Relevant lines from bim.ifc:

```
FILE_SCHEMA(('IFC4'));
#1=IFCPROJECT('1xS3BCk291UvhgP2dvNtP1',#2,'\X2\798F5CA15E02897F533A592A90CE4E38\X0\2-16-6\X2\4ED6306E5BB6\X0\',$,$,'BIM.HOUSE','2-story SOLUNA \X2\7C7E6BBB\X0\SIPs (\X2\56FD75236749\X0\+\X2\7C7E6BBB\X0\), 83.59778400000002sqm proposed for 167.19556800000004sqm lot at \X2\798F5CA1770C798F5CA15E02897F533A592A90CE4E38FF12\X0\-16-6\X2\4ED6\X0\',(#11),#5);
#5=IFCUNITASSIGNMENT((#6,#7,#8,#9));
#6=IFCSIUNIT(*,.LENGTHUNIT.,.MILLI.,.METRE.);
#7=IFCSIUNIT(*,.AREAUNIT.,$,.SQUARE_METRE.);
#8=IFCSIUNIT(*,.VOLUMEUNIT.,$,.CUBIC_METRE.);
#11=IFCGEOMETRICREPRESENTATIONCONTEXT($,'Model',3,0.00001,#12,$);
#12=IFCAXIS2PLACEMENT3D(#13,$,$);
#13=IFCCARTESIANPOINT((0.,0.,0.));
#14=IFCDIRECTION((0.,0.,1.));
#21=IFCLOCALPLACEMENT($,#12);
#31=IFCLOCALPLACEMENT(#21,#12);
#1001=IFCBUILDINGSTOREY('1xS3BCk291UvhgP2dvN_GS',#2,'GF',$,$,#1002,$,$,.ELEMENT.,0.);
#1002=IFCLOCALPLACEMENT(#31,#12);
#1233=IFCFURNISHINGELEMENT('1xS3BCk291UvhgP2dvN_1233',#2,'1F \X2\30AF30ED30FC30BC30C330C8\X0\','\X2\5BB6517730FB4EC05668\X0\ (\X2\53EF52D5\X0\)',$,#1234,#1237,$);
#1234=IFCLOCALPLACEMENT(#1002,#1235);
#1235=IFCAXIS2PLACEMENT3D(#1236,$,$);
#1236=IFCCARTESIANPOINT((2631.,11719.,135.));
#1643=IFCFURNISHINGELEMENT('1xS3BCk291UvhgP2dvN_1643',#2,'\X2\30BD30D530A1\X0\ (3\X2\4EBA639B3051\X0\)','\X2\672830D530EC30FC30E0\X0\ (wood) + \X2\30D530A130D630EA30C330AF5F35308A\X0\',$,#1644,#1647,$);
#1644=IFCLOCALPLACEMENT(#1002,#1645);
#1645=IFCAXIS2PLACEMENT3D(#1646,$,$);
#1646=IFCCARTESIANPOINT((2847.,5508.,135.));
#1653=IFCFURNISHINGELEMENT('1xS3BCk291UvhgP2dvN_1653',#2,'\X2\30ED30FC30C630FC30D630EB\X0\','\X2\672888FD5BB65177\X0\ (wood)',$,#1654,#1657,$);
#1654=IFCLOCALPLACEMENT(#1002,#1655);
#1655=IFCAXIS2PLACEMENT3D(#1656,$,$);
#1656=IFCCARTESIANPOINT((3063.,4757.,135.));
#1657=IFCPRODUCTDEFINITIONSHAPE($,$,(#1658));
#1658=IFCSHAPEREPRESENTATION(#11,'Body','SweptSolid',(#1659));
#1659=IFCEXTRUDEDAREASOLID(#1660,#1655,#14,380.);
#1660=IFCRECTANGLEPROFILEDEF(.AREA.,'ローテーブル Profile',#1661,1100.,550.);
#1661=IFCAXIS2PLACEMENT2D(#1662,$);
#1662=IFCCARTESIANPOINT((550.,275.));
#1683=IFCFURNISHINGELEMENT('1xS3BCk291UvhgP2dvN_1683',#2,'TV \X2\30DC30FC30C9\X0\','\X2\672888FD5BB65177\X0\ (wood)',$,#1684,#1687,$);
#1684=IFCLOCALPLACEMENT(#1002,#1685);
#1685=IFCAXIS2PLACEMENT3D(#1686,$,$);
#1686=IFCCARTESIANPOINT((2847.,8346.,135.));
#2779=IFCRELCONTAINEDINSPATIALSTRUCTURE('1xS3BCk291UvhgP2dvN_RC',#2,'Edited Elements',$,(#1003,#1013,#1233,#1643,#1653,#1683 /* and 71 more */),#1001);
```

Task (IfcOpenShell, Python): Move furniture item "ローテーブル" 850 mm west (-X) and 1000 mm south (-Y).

```python
import ifcopenshell
import ifcopenshell.api.geometry
import ifcopenshell.util.placement
import ifcopenshell.util.unit

model = ifcopenshell.open("bim.ifc")
unit_scale = ifcopenshell.util.unit.calculate_unit_scale(model)

item = model.by_guid("1xS3BCk291UvhgP2dvN_1653")
matrix = ifcopenshell.util.placement.get_local_placement(item.ObjectPlacement)
matrix[0, 3] -= 0.85 / unit_scale
matrix[1, 3] -= 1 / unit_scale
ifcopenshell.api.geometry.edit_object_placement(model, product=item, matrix=matrix, is_si=False)

print(ifcopenshell.util.placement.get_local_placement(item.ObjectPlacement).round(3) + 0.0)

model.write("bim_v2.ifc")
```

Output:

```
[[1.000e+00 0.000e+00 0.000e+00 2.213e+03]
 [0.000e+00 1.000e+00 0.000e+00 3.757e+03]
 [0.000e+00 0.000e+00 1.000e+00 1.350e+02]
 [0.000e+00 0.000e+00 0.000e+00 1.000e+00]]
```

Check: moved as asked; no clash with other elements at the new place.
